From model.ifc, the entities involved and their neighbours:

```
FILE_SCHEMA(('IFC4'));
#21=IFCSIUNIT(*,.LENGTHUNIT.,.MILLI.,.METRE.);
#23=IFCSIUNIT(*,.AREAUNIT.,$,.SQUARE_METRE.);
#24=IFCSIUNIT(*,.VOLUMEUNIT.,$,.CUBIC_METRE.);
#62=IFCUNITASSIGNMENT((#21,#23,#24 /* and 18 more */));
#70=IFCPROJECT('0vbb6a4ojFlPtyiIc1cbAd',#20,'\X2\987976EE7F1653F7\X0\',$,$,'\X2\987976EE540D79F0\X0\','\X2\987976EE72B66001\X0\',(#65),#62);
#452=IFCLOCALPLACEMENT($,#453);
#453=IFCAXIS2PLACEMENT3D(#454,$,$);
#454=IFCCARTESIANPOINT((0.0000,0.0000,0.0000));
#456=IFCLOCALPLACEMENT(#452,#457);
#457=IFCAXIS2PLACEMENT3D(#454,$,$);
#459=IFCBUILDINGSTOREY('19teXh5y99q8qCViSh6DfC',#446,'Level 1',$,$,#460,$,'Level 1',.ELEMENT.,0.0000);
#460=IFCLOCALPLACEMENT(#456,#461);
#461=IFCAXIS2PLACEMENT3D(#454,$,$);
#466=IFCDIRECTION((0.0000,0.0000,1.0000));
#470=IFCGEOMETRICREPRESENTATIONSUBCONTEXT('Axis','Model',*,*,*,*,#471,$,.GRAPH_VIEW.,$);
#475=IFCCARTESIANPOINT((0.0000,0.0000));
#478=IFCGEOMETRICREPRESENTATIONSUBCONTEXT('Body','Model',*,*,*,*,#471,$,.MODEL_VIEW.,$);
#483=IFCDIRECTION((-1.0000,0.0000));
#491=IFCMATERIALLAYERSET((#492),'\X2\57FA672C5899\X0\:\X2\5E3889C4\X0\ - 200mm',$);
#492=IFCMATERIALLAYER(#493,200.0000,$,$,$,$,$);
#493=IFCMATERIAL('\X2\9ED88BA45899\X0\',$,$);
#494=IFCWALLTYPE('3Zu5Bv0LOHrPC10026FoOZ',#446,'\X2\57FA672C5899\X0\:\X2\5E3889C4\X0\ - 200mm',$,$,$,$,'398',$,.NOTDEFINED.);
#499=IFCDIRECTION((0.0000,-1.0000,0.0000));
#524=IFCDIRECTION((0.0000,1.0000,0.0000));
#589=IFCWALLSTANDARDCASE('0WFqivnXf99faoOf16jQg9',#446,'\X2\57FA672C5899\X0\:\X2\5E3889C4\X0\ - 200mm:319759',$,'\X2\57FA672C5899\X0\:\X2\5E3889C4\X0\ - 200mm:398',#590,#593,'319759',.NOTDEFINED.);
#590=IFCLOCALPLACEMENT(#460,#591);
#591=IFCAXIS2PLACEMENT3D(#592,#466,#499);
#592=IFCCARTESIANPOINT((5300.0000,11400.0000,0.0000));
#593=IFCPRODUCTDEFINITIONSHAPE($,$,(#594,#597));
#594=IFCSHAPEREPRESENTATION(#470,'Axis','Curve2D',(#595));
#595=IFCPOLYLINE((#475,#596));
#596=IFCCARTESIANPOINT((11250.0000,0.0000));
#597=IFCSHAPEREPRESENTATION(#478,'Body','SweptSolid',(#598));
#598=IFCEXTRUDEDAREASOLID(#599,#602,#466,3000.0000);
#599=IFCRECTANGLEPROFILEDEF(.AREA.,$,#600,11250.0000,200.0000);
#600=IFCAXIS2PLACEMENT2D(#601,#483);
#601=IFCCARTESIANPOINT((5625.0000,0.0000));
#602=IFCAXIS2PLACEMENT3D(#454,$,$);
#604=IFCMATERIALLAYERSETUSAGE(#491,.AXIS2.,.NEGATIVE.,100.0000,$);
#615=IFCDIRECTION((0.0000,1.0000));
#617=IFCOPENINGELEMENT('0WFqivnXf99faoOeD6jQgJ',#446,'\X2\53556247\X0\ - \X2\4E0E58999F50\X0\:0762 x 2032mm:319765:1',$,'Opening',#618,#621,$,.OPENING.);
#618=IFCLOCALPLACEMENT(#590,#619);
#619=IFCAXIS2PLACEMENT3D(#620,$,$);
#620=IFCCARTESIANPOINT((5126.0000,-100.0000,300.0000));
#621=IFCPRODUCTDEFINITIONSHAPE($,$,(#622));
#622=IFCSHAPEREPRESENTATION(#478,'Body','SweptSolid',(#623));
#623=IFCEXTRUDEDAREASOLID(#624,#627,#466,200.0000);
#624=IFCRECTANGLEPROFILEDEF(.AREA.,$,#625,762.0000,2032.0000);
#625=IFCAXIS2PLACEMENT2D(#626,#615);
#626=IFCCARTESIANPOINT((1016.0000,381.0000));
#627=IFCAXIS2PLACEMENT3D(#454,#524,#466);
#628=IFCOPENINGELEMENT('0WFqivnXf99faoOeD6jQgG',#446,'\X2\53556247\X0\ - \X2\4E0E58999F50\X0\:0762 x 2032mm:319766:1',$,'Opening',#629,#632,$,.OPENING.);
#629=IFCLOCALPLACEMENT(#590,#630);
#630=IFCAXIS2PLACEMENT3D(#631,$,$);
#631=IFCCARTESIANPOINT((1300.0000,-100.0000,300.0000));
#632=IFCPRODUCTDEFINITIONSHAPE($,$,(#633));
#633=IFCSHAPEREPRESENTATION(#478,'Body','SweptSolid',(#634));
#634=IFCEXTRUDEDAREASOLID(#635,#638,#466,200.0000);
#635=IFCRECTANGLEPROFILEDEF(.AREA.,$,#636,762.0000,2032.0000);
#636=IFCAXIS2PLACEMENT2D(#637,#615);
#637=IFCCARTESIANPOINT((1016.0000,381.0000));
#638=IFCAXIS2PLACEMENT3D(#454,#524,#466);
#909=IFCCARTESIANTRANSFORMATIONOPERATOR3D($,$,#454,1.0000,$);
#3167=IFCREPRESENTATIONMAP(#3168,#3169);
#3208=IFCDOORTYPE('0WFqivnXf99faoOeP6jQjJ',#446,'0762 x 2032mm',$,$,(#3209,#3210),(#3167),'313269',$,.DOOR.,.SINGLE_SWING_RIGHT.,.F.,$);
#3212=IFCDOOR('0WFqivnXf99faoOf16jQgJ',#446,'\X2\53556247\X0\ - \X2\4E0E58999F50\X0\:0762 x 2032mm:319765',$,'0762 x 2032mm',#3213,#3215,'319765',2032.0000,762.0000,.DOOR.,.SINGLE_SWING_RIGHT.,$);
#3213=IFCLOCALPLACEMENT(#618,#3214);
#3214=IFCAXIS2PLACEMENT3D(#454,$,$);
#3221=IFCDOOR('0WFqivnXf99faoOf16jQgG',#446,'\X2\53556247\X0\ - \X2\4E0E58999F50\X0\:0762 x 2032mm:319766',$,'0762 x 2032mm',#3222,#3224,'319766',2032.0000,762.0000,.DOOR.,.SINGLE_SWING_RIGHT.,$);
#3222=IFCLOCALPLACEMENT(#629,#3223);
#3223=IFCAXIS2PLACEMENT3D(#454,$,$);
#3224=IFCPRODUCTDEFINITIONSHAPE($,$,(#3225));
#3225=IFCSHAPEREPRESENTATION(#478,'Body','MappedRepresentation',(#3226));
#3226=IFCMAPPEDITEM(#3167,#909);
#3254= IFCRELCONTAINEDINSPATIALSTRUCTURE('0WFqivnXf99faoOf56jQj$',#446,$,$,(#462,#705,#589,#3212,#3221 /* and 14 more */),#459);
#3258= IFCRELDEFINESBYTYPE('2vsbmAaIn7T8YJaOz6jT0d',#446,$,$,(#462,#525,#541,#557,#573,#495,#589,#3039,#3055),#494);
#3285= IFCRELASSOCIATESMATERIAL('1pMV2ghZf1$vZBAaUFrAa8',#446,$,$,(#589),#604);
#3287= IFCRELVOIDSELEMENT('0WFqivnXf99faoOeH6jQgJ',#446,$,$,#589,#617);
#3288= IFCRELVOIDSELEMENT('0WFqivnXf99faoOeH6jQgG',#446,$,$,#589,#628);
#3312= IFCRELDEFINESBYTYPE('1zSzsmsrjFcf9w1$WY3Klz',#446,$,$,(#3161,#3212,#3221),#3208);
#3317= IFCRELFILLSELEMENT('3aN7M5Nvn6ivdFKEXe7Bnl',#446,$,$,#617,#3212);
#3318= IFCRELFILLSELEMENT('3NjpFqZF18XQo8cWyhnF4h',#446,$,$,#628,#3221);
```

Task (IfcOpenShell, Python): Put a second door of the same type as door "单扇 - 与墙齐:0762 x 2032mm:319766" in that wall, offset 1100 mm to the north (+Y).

```python
import ifcopenshell
import ifcopenshell.api.feature
import ifcopenshell.api.geometry
import ifcopenshell.api.root
import ifcopenshell.geom
import ifcopenshell.util.element
import ifcopenshell.util.placement
import ifcopenshell.util.shape

model = ifcopenshell.open("model.ifc")
settings = ifcopenshell.geom.settings()


def volume(element):
    """Net volume in cubic metres, openings subtracted."""
    shape = ifcopenshell.geom.create_shape(settings, element)
    return ifcopenshell.util.shape.get_volume(shape.geometry)


def reuse_history(source, copy):
    """copy_class also copies each property set's owner history, people and application; keep the originals."""
    for rel in copy.IsDefinedBy:
        if rel.is_a("IfcRelDefinesByProperties") and (history := rel.RelatingPropertyDefinition.OwnerHistory):
            rel.RelatingPropertyDefinition.OwnerHistory = source.OwnerHistory
            ifcopenshell.util.element.remove_deep2(model, history)


door = model.by_guid("0WFqivnXf99faoOf16jQgG")
opening = door.FillsVoids[0].RelatingOpeningElement
wall = opening.VoidsElements[0].RelatingBuildingElement
before = volume(wall)
shift = ifcopenshell.util.placement.get_local_placement(wall.ObjectPlacement)[:3, 0] * -1100.0

# copy_class copies the void relationship, type, container and properties, but no geometry.
new_opening = ifcopenshell.api.root.copy_class(model, product=opening)
new_opening.Representation = ifcopenshell.util.element.copy_deep(
    model, opening.Representation, exclude=["IfcGeometricRepresentationContext", "IfcRepresentationMap"]
)
new_opening.Name = "单扇 - 与墙齐:0762 x 2032mm"
new_door = ifcopenshell.api.root.copy_class(model, product=door)
new_door.Representation = ifcopenshell.util.element.copy_deep(
    model, door.Representation, exclude=["IfcGeometricRepresentationContext", "IfcRepresentationMap"]
)
new_door.Name = "单扇 - 与墙齐:0762 x 2032mm"
new_door.Tag = None
reuse_history(door, new_door)
ifcopenshell.api.feature.add_filling(model, opening=new_opening, element=new_door)

for old, new in ((opening, new_opening), (door, new_door)):
    matrix = ifcopenshell.util.placement.get_local_placement(old.ObjectPlacement)
    matrix[:3, 3] += shift
    ifcopenshell.api.geometry.edit_object_placement(model, product=new, matrix=matrix, is_si=False)

after = volume(wall)

print(f"wall volume {before:.3f} -> {after:.3f} m3")

model.write("model_rev.ifc")
```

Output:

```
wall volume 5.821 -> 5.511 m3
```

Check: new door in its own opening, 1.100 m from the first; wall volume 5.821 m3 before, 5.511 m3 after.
